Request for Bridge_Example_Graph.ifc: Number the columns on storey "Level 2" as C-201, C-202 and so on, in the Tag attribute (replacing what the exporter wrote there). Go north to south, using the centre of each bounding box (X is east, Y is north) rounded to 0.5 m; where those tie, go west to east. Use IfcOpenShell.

First a look at what the model holds.

```python
import ifcopenshell
import ifcopenshell.util.element
import ifcopenshell.util.placement

model = ifcopenshell.open("Bridge_Example_Graph.ifc")
print(model.schema)
storey = next(s for s in model.by_type("IfcBuildingStorey") if s.Name == "Level 2")
columns = [e for e in ifcopenshell.util.element.get_decomposition(storey) if e.is_a("IfcColumn")]
for e in sorted(columns, key=lambda e: e.id()):
    origin = ifcopenshell.util.placement.get_local_placement(e.ObjectPlacement)[:3, 3]
    print(e.id(), e.Tag, e.Name, origin.round(2) + 0.0, sep=" | ")
```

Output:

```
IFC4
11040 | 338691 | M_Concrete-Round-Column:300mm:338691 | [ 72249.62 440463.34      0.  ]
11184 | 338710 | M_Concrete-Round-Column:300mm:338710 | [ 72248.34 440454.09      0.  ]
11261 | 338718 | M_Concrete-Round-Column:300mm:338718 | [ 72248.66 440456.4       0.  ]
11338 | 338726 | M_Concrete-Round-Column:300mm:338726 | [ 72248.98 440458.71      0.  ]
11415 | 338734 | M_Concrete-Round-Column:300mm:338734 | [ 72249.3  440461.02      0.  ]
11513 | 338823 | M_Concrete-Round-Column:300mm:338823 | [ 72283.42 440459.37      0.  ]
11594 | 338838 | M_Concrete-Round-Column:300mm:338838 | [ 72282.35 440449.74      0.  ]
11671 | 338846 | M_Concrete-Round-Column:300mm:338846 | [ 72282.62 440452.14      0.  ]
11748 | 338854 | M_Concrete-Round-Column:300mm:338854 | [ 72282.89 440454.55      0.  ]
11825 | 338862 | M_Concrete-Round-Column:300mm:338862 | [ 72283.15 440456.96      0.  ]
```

```python
import ifcopenshell
import ifcopenshell.geom
import ifcopenshell.util.element
import ifcopenshell.util.shape

model = ifcopenshell.open("Bridge_Example_Graph.ifc")
settings = ifcopenshell.geom.settings()
settings.set("use-world-coords", True)


def centre(element):
    shape = ifcopenshell.geom.create_shape(settings, element)
    return ifcopenshell.util.shape.get_bbox_centroid(shape.geometry)


storey = next(s for s in model.by_type("IfcBuildingStorey") if s.Name == "Level 2")
columns = [e for e in ifcopenshell.util.element.get_decomposition(storey) if e.is_a("IfcColumn")]

# Insertion points can sit at a corner or the storey origin, so sort by the geometry (in metres).
centres = {e: centre(e) for e in columns}
columns.sort(key=lambda e: (-round(centres[e][1] / 0.5), centres[e][0]))

for i, e in enumerate(columns, start=1):
    number = f"C-2{i:02d}"
    e.Tag = number
    print(e.id(), number)

model.write("Bridge_Example_Graph_updated.ifc")
```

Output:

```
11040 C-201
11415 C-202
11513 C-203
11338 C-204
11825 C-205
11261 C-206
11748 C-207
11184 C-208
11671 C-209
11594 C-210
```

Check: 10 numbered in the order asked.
